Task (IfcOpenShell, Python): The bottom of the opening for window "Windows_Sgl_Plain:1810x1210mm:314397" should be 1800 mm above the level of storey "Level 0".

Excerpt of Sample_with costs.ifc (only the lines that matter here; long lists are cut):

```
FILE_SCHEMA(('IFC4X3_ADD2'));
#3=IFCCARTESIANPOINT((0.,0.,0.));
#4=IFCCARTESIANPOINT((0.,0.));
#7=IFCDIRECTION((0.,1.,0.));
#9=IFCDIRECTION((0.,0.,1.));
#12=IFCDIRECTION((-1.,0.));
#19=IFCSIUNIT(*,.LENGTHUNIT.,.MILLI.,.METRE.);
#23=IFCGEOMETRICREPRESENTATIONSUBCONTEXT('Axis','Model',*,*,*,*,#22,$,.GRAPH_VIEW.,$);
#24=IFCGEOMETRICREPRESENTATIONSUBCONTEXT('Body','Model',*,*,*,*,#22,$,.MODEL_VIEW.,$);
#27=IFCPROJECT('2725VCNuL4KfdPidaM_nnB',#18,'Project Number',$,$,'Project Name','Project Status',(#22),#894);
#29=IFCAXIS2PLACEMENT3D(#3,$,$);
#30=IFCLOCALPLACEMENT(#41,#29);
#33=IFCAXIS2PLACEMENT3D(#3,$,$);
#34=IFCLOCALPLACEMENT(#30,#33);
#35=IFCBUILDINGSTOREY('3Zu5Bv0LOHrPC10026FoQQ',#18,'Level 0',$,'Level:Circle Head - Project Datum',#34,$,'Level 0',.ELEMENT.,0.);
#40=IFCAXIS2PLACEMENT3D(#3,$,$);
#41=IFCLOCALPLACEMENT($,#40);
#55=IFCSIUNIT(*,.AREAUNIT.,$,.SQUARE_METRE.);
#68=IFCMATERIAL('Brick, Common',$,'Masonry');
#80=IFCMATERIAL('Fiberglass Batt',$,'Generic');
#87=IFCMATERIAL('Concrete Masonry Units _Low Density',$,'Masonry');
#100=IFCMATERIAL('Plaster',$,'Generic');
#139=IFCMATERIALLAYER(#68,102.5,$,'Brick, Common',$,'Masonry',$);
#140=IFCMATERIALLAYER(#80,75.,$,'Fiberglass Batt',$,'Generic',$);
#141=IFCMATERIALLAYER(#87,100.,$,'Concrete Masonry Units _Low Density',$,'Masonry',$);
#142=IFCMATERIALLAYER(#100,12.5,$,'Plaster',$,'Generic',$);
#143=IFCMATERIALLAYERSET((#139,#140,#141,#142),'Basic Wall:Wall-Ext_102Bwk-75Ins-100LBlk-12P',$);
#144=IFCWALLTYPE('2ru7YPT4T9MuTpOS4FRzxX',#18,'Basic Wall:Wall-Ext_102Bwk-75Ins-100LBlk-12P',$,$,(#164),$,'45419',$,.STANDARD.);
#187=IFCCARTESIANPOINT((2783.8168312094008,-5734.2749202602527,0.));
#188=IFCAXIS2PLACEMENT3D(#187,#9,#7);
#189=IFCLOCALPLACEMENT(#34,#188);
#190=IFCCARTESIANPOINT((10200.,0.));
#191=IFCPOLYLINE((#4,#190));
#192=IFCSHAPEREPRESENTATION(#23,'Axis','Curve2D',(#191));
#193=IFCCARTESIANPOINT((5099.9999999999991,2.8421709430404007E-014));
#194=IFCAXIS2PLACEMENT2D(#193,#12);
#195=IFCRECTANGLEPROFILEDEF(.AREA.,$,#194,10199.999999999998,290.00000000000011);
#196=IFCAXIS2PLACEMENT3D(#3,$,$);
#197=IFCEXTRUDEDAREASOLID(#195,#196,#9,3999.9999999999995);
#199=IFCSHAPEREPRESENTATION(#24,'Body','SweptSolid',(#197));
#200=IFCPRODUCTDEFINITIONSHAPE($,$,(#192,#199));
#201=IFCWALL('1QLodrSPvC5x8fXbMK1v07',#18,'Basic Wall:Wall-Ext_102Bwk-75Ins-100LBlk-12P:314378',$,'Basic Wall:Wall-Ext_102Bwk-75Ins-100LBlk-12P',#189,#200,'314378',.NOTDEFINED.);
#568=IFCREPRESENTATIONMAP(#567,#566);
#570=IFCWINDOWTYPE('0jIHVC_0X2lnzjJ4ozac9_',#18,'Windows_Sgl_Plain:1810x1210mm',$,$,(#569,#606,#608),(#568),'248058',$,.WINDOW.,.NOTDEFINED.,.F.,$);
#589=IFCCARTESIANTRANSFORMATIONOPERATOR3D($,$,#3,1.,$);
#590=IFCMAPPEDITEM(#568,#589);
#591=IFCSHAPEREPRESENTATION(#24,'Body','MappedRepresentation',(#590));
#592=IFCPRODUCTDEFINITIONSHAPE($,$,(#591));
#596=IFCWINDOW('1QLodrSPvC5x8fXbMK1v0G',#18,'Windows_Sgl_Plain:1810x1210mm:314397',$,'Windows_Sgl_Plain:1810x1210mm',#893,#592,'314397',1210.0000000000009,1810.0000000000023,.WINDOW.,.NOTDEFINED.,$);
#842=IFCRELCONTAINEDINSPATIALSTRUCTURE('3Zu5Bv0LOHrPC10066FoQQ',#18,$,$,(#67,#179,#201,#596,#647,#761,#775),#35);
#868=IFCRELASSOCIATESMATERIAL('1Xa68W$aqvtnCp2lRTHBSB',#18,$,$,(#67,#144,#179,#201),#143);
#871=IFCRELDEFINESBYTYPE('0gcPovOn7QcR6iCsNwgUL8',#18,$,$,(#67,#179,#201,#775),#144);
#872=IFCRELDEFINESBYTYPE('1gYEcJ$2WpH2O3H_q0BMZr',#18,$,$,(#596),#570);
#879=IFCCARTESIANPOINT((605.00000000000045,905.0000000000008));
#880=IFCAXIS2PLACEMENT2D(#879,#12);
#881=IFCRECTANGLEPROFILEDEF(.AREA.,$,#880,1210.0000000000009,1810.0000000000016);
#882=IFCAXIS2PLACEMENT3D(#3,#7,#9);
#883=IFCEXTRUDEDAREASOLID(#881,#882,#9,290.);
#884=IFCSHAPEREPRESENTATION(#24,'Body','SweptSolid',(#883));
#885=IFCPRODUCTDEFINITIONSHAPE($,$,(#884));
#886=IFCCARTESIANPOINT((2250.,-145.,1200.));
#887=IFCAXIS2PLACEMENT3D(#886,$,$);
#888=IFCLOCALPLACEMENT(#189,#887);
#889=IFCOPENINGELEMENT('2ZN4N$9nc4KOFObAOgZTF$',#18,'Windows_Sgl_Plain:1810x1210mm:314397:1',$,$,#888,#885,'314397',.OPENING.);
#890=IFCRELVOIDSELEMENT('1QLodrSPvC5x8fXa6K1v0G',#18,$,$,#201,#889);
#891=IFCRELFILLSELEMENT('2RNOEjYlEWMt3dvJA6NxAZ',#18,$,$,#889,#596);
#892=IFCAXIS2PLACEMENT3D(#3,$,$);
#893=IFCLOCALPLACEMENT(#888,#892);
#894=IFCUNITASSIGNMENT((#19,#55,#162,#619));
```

```python
import numpy as np
import ifcopenshell
import ifcopenshell.api.geometry
import ifcopenshell.geom
import ifcopenshell.util.element
import ifcopenshell.util.placement
import ifcopenshell.util.shape
import ifcopenshell.util.unit

model = ifcopenshell.open("Sample_with costs.ifc")
unit_scale = ifcopenshell.util.unit.calculate_unit_scale(model)

window = model.by_id(596)
opening = window.FillsVoids[0].RelatingOpeningElement
storey = ifcopenshell.util.element.get_container(window, ifc_class="IfcBuildingStorey")
level = ifcopenshell.util.placement.get_local_placement(storey.ObjectPlacement)[2, 3]

# The opening's origin need not be at the sill, so measure its lowest point.
shape = ifcopenshell.geom.create_shape(ifcopenshell.geom.settings(), opening)
bottom = ifcopenshell.util.shape.get_shape_bottom_elevation(shape, shape.geometry) / unit_scale
dz = level + 1.8 / unit_scale - bottom

shift = np.array([0.0, 0.0, dz])
# The window is placed relative to its opening, so it follows when the opening moves.
matrix = ifcopenshell.util.placement.get_local_placement(opening.ObjectPlacement)
matrix[:3, 3] += shift
ifcopenshell.api.geometry.edit_object_placement(
    model, product=opening, matrix=matrix, is_si=False, should_transform_children=True
)

print(f"moved by {dz * unit_scale:+.3f} m")

model.write("Sample_with costs_rev.ifc")
```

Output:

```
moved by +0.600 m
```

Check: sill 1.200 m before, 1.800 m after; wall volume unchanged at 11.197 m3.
